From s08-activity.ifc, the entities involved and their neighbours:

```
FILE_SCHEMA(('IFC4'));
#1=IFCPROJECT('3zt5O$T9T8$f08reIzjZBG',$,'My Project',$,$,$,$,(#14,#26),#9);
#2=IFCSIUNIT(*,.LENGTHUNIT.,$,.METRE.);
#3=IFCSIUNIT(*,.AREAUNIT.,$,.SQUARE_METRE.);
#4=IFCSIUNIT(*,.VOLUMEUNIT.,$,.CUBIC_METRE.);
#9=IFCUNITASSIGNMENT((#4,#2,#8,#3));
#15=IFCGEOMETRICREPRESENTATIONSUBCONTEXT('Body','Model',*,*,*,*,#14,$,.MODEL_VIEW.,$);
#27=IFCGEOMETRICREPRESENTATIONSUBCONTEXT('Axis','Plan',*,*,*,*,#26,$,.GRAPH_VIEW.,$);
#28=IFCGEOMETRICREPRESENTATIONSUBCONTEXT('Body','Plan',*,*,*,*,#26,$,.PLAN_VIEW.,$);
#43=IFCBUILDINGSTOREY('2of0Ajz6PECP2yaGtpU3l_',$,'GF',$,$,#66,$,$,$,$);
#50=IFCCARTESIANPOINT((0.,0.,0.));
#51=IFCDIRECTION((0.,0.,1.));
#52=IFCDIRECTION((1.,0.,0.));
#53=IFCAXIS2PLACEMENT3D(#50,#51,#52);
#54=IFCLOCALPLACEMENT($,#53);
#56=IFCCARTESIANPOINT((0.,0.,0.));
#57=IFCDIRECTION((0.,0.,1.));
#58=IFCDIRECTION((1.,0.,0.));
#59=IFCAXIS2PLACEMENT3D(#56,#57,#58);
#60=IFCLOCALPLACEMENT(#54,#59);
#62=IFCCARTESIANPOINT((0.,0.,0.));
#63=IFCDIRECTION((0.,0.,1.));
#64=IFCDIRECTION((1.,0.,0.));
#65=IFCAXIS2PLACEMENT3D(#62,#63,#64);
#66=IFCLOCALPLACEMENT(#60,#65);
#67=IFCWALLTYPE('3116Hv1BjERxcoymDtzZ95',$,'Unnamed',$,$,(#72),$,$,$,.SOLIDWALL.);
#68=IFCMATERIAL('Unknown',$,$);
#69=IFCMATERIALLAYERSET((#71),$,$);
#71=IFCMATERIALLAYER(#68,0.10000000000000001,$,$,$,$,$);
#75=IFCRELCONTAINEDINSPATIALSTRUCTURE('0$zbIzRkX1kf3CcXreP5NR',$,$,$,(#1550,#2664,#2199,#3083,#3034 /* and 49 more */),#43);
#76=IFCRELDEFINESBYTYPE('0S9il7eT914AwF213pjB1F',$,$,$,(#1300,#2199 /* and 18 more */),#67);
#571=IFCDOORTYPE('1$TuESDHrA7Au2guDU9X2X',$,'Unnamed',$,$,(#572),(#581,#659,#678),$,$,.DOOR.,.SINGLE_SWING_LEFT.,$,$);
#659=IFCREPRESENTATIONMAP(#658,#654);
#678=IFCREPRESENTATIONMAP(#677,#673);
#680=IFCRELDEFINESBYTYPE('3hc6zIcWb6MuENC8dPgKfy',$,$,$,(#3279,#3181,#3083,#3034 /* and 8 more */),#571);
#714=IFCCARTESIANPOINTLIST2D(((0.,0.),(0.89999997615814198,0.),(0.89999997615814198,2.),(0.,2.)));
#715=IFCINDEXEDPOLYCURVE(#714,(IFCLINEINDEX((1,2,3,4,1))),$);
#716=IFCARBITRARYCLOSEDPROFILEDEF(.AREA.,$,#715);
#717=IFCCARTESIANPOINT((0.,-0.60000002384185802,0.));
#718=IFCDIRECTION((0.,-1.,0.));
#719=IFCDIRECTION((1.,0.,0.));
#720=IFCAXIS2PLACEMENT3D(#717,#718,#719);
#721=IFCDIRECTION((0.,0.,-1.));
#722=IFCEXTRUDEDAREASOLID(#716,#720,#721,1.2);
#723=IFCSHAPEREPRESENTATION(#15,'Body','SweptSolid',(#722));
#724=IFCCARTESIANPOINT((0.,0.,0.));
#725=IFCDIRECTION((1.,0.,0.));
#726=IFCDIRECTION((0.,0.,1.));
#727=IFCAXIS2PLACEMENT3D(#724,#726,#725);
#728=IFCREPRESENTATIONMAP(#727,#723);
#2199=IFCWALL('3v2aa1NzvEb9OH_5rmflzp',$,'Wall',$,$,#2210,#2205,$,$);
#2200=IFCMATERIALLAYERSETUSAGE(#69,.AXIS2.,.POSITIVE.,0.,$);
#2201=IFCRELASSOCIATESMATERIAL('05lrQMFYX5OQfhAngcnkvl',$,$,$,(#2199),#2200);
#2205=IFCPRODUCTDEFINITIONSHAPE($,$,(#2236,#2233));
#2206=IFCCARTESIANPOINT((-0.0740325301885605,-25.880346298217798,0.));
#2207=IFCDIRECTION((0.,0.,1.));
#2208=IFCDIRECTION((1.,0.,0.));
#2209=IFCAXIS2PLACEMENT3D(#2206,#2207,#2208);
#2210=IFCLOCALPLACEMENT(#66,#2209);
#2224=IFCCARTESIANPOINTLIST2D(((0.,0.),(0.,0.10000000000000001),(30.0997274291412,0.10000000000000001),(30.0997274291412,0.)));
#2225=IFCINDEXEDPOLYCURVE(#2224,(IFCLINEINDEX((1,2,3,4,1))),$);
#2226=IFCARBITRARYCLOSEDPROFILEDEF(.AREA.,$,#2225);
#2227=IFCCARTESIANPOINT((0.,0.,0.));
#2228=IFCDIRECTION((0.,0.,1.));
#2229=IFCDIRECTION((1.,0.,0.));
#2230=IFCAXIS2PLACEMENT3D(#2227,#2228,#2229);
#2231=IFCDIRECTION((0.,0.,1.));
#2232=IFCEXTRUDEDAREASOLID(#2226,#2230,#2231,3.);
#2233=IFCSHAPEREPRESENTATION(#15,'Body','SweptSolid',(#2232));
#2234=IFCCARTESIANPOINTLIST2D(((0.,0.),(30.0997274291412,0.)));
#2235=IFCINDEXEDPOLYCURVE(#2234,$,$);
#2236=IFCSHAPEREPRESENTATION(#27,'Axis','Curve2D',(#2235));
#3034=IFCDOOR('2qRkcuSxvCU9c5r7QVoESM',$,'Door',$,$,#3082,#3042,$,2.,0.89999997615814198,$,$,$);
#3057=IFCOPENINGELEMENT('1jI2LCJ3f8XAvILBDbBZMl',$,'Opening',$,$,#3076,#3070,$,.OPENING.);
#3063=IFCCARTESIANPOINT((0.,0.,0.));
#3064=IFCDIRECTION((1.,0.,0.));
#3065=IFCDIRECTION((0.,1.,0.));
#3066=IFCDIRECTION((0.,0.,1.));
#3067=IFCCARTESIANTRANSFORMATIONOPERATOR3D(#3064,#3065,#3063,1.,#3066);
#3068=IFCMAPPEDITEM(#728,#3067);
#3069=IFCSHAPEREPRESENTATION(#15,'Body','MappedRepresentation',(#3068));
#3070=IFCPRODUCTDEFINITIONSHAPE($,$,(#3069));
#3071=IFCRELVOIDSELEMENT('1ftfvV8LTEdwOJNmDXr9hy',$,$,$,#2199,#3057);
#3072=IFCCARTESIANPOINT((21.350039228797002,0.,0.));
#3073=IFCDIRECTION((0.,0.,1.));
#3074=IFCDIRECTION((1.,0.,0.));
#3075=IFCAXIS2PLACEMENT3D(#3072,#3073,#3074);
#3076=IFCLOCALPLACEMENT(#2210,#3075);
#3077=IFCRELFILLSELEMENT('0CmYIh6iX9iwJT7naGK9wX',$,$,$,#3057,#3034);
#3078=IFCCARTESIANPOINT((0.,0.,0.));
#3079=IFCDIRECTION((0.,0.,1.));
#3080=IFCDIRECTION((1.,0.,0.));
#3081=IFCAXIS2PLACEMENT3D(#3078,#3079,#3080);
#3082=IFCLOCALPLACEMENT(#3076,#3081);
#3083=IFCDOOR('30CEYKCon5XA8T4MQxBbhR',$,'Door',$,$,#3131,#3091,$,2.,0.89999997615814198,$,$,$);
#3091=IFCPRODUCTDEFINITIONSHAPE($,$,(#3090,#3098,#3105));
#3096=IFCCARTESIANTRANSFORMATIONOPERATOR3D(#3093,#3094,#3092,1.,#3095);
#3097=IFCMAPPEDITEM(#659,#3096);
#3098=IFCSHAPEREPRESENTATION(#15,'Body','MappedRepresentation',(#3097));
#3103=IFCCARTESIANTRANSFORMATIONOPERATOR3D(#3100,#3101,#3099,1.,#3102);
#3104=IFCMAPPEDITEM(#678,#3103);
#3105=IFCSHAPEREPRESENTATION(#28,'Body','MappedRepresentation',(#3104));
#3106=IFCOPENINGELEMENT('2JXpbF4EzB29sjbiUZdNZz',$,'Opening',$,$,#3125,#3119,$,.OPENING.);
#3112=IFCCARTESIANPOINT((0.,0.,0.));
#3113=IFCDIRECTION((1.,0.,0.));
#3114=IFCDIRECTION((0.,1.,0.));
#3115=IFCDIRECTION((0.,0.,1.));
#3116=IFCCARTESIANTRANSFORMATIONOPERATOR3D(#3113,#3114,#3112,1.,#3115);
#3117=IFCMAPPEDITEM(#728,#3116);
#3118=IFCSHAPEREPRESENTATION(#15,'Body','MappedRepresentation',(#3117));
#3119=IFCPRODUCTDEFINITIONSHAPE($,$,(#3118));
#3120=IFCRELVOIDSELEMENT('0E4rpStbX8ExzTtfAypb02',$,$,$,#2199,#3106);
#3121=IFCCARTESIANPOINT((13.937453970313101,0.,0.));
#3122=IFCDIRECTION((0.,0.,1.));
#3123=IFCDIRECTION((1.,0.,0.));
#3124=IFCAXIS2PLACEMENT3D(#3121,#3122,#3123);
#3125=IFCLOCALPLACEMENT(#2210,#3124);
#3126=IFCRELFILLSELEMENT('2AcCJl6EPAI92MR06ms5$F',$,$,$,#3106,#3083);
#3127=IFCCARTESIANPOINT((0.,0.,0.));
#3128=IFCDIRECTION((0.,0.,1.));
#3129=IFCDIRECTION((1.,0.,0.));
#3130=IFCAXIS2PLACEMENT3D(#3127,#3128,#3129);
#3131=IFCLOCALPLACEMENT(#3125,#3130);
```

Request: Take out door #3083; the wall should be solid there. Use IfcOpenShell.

```python
import ifcopenshell
import ifcopenshell.api.feature
import ifcopenshell.api.root
import ifcopenshell.geom
import ifcopenshell.util.shape

model = ifcopenshell.open("s08-activity.ifc")
settings = ifcopenshell.geom.settings()


def volume(element):
    """Net volume in cubic metres, openings subtracted."""
    shape = ifcopenshell.geom.create_shape(settings, element)
    return ifcopenshell.util.shape.get_volume(shape.geometry)


door = model.by_guid("30CEYKCon5XA8T4MQxBbhR")
opening = door.FillsVoids[0].RelatingOpeningElement
wall = opening.VoidsElements[0].RelatingBuildingElement
before = volume(wall)

ifcopenshell.api.root.remove_product(model, product=door)
ifcopenshell.api.feature.remove_feature(model, feature=opening)

after = volume(wall)

print(f"wall volume {before:.3f} -> {after:.3f} m3")

model.write("s08-activity_v2.ifc")
```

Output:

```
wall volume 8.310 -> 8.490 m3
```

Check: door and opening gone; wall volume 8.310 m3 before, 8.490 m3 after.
